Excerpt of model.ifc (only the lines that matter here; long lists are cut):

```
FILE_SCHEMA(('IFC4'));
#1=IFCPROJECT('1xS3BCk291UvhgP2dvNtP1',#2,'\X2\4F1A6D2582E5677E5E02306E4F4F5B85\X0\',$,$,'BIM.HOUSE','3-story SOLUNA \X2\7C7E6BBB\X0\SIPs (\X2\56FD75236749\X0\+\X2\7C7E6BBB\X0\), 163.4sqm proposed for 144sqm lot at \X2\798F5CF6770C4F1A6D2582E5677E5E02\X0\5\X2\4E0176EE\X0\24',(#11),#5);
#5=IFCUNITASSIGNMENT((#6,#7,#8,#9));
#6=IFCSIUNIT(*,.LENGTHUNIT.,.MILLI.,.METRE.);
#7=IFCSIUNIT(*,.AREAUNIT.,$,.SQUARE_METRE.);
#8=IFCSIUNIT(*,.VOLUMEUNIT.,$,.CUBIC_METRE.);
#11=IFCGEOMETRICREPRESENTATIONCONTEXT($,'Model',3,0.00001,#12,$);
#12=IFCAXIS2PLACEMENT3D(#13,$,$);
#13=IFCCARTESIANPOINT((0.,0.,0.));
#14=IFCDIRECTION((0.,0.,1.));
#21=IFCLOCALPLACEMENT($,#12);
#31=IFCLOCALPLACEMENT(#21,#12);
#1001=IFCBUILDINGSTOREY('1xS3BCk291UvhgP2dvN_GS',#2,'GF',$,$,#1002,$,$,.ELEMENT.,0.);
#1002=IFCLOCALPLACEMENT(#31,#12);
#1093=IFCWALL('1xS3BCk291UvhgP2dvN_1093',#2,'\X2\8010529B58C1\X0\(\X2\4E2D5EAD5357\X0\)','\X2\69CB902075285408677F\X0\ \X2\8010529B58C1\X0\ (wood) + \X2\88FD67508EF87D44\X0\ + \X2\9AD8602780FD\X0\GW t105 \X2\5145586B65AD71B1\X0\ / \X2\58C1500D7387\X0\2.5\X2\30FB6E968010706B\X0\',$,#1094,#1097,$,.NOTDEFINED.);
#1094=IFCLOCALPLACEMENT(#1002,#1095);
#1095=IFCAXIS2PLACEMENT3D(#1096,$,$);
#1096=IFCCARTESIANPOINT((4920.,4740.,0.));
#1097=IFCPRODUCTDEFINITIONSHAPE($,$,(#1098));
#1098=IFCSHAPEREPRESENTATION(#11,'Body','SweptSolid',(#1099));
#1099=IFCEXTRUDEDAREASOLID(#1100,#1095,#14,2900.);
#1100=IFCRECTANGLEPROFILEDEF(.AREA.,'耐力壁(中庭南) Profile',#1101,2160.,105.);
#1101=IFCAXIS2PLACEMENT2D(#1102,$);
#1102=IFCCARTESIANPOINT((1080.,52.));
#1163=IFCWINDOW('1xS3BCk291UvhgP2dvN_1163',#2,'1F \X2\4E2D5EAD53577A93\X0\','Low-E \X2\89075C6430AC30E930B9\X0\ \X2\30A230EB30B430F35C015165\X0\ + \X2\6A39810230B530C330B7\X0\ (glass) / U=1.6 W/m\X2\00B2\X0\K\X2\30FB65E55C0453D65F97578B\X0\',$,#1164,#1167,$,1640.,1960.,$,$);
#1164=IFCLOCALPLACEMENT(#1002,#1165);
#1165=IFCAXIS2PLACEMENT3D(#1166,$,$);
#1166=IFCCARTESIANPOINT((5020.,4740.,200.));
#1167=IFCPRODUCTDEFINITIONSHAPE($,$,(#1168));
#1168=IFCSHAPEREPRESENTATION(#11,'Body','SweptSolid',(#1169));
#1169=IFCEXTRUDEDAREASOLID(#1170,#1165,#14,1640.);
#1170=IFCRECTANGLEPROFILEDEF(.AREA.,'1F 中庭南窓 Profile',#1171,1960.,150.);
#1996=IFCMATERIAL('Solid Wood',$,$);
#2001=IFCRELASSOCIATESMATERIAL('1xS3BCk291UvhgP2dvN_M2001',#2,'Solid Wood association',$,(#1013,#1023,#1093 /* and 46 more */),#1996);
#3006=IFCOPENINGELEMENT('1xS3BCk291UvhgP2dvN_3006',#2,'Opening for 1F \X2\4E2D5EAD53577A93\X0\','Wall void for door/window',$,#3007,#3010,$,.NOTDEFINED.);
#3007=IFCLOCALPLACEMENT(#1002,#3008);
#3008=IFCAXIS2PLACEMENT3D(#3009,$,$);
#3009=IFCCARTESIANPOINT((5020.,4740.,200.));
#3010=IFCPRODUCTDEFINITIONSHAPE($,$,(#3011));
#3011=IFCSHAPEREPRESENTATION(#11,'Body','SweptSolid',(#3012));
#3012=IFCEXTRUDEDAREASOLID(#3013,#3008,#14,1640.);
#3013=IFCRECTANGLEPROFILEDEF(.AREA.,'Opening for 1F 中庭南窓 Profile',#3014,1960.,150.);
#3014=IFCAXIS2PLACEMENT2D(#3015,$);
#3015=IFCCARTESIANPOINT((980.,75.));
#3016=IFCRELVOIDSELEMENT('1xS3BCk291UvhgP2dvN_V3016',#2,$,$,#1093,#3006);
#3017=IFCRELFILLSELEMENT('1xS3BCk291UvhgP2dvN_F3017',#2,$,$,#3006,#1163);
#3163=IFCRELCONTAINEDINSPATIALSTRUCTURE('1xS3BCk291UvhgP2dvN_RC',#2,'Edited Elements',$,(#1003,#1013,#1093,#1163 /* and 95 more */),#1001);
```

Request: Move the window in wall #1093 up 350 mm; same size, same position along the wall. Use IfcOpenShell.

```python
import numpy as np
import ifcopenshell
import ifcopenshell.api.geometry
import ifcopenshell.util.placement
import ifcopenshell.util.unit

model = ifcopenshell.open("model.ifc")
unit_scale = ifcopenshell.util.unit.calculate_unit_scale(model)

window = model.by_id(1163)
opening = window.FillsVoids[0].RelatingOpeningElement
dz = 0.35 / unit_scale

shift = np.array([0.0, 0.0, dz])
# The window is not placed relative to its opening, so move both.
for product in (opening, window):
    matrix = ifcopenshell.util.placement.get_local_placement(product.ObjectPlacement)
    matrix[:3, 3] += shift
    ifcopenshell.api.geometry.edit_object_placement(model, product=product, matrix=matrix, is_si=False)

print(f"moved by {dz * unit_scale:+.3f} m")

model.write("model_updated.ifc")
```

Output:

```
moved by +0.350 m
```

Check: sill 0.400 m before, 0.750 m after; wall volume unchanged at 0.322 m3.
